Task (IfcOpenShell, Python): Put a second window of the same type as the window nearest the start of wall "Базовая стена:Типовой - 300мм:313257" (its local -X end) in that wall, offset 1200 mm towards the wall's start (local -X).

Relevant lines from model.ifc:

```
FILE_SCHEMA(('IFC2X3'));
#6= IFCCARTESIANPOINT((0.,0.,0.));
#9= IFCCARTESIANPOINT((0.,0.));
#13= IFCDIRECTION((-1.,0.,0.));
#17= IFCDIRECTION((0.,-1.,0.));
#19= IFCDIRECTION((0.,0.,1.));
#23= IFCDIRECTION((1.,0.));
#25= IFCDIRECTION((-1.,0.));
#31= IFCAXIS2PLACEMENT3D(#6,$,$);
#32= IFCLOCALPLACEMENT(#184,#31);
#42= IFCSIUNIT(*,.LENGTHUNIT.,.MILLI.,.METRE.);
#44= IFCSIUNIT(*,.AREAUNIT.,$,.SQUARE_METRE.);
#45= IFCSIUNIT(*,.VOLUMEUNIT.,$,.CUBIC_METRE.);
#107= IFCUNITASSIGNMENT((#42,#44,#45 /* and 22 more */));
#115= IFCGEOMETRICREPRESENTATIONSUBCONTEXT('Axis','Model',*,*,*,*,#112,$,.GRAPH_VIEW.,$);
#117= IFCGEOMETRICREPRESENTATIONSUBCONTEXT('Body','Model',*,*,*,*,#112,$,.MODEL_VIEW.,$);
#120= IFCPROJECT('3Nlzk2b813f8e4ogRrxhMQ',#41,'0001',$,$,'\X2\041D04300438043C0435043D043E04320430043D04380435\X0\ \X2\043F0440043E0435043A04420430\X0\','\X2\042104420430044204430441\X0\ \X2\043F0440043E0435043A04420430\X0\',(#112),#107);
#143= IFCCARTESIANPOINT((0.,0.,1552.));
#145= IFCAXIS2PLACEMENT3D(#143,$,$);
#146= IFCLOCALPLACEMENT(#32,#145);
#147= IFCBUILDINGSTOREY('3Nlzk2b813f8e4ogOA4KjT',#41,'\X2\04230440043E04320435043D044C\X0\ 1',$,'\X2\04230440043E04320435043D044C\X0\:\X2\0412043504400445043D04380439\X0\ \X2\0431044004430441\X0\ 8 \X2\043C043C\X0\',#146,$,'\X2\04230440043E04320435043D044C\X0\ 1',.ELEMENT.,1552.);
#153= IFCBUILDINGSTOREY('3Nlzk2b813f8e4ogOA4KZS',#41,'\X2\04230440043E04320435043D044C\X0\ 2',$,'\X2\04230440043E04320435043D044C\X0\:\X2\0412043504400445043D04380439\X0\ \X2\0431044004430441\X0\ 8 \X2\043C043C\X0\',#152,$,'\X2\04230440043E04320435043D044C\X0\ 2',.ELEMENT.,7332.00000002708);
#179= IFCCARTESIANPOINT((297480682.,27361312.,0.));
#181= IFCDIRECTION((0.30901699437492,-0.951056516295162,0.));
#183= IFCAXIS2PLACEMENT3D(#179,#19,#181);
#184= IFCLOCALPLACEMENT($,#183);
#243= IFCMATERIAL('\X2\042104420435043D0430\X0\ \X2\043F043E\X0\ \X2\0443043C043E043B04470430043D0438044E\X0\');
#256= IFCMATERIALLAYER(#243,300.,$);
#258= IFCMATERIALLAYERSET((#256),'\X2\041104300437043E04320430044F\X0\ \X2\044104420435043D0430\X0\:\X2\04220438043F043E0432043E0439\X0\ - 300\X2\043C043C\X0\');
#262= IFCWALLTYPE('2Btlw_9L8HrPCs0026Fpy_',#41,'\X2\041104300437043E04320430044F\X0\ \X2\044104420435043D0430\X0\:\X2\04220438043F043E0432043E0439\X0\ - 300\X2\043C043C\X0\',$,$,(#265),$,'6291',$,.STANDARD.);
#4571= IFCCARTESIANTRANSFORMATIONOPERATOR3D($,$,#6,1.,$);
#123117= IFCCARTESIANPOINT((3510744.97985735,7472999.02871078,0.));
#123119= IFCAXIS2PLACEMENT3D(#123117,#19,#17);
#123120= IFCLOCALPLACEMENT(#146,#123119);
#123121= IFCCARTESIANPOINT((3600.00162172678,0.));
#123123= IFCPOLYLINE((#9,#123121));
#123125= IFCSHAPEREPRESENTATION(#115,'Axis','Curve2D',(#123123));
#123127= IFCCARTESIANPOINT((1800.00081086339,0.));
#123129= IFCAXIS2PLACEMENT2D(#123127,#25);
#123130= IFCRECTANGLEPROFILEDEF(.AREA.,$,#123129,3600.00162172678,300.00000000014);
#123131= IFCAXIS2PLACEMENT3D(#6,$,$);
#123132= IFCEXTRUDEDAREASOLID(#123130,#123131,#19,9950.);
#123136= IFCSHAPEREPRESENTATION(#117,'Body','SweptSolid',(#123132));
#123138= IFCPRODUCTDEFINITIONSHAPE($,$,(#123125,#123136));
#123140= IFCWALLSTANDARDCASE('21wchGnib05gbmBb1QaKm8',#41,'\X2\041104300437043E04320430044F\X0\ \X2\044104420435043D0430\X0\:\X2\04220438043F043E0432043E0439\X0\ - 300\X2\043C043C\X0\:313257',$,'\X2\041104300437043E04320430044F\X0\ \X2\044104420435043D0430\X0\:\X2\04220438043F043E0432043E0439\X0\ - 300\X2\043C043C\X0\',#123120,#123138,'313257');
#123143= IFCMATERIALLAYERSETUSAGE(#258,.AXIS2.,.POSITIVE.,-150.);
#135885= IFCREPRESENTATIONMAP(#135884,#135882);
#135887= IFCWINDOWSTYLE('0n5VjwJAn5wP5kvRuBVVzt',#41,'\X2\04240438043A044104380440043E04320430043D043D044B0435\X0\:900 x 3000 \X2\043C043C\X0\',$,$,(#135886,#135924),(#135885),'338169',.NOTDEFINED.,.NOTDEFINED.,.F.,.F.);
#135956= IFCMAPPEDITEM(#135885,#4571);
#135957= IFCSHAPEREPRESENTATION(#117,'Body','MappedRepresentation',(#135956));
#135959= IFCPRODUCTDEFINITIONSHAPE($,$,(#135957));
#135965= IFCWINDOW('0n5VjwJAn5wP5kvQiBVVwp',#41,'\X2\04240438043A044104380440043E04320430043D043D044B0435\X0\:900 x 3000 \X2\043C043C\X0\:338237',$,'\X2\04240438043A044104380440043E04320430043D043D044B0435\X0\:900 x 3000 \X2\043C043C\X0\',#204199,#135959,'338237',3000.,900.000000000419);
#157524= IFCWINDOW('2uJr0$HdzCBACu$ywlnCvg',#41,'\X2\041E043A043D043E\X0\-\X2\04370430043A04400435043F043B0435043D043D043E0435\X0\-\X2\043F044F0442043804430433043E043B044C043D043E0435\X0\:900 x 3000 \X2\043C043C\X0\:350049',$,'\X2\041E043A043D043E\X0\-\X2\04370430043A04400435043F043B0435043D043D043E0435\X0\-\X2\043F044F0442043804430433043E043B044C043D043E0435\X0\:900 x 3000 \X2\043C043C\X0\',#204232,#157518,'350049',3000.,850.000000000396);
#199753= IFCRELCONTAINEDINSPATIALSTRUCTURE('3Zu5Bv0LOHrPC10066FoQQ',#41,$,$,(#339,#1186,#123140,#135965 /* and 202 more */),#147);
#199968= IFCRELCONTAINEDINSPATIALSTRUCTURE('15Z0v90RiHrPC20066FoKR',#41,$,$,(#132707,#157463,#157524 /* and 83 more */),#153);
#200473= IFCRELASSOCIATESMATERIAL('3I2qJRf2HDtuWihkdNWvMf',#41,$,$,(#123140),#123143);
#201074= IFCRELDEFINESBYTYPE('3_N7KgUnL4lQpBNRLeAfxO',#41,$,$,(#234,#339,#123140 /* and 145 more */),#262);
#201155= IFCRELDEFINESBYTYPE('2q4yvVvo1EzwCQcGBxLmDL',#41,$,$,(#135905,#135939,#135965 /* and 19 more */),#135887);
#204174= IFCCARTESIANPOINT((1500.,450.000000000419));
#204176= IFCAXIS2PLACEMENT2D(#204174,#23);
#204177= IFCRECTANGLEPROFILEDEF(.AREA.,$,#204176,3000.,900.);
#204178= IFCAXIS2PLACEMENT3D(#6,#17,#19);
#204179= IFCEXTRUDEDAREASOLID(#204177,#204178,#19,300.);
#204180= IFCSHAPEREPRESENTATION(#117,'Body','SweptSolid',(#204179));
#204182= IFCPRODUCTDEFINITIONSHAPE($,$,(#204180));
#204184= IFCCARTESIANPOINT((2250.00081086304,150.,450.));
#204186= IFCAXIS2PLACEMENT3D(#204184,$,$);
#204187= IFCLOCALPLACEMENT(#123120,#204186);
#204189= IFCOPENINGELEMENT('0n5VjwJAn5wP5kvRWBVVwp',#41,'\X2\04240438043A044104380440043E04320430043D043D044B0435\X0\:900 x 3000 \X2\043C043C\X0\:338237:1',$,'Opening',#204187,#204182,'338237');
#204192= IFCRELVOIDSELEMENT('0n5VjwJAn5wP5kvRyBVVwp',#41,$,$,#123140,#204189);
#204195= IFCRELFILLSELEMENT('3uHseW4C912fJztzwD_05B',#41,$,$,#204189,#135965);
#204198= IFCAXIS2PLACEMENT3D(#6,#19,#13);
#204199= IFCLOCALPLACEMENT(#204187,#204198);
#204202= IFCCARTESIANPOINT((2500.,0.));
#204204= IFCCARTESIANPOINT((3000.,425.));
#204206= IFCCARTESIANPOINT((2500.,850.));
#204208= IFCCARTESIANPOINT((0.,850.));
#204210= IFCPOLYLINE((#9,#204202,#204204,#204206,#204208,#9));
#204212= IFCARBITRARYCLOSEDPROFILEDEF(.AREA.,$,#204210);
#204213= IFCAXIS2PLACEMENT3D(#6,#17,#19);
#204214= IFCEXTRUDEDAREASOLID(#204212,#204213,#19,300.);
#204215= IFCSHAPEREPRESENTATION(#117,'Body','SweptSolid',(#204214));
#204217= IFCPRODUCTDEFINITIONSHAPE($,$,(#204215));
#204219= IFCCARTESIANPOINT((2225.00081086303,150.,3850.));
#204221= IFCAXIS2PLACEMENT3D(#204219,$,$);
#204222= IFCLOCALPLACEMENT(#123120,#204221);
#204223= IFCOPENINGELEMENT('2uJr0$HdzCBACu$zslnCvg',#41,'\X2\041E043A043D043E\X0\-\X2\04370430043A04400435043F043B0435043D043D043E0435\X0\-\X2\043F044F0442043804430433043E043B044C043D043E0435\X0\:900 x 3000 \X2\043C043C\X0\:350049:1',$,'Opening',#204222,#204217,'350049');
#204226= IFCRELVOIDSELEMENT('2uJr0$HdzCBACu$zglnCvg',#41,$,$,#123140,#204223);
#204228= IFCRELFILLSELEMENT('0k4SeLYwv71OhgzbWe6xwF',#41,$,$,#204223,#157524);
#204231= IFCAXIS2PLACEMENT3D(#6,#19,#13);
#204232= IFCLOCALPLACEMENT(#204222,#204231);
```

```python
import ifcopenshell
import ifcopenshell.api.feature
import ifcopenshell.api.geometry
import ifcopenshell.api.root
import ifcopenshell.geom
import ifcopenshell.util.element
import ifcopenshell.util.placement
import ifcopenshell.util.shape

model = ifcopenshell.open("model.ifc")
settings = ifcopenshell.geom.settings()


def volume(element):
    """Net volume in cubic metres, openings subtracted."""
    shape = ifcopenshell.geom.create_shape(settings, element)
    return ifcopenshell.util.shape.get_volume(shape.geometry)


def reuse_history(source, copy):
    """copy_class also copies each property set's owner history, people and application; keep the originals."""
    for rel in copy.IsDefinedBy:
        if rel.is_a("IfcRelDefinesByProperties") and (history := rel.RelatingPropertyDefinition.OwnerHistory):
            rel.RelatingPropertyDefinition.OwnerHistory = source.OwnerHistory
            ifcopenshell.util.element.remove_deep2(model, history)


window = model.by_id(135965)
opening = window.FillsVoids[0].RelatingOpeningElement
wall = opening.VoidsElements[0].RelatingBuildingElement
before = volume(wall)
shift = ifcopenshell.util.placement.get_local_placement(wall.ObjectPlacement)[:3, 0] * -1200.0

# copy_class copies the void relationship, type, container and properties, but no geometry.
new_opening = ifcopenshell.api.root.copy_class(model, product=opening)
new_opening.Representation = ifcopenshell.util.element.copy_deep(
    model, opening.Representation, exclude=["IfcGeometricRepresentationContext", "IfcRepresentationMap"]
)
new_opening.Name = "Фиксированные:900 x 3000 мм"
new_opening.Tag = None
new_window = ifcopenshell.api.root.copy_class(model, product=window)
new_window.Representation = ifcopenshell.util.element.copy_deep(
    model, window.Representation, exclude=["IfcGeometricRepresentationContext", "IfcRepresentationMap"]
)
new_window.Name = "Фиксированные:900 x 3000 мм"
new_window.Tag = None
reuse_history(window, new_window)
fills = ifcopenshell.api.feature.add_filling(model, opening=new_opening, element=new_window)
fills.OwnerHistory = new_window.OwnerHistory  # required in IFC2X3

for old, new in ((opening, new_opening), (window, new_window)):
    matrix = ifcopenshell.util.placement.get_local_placement(old.ObjectPlacement)
    matrix[:3, 3] += shift
    ifcopenshell.api.geometry.edit_object_placement(model, product=new, matrix=matrix, is_si=False)

after = volume(wall)

print(f"wall volume {before:.3f} -> {after:.3f} m3")

model.write("model_v2.ifc")
```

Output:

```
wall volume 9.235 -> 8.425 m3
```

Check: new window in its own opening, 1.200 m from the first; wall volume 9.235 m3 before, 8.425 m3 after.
